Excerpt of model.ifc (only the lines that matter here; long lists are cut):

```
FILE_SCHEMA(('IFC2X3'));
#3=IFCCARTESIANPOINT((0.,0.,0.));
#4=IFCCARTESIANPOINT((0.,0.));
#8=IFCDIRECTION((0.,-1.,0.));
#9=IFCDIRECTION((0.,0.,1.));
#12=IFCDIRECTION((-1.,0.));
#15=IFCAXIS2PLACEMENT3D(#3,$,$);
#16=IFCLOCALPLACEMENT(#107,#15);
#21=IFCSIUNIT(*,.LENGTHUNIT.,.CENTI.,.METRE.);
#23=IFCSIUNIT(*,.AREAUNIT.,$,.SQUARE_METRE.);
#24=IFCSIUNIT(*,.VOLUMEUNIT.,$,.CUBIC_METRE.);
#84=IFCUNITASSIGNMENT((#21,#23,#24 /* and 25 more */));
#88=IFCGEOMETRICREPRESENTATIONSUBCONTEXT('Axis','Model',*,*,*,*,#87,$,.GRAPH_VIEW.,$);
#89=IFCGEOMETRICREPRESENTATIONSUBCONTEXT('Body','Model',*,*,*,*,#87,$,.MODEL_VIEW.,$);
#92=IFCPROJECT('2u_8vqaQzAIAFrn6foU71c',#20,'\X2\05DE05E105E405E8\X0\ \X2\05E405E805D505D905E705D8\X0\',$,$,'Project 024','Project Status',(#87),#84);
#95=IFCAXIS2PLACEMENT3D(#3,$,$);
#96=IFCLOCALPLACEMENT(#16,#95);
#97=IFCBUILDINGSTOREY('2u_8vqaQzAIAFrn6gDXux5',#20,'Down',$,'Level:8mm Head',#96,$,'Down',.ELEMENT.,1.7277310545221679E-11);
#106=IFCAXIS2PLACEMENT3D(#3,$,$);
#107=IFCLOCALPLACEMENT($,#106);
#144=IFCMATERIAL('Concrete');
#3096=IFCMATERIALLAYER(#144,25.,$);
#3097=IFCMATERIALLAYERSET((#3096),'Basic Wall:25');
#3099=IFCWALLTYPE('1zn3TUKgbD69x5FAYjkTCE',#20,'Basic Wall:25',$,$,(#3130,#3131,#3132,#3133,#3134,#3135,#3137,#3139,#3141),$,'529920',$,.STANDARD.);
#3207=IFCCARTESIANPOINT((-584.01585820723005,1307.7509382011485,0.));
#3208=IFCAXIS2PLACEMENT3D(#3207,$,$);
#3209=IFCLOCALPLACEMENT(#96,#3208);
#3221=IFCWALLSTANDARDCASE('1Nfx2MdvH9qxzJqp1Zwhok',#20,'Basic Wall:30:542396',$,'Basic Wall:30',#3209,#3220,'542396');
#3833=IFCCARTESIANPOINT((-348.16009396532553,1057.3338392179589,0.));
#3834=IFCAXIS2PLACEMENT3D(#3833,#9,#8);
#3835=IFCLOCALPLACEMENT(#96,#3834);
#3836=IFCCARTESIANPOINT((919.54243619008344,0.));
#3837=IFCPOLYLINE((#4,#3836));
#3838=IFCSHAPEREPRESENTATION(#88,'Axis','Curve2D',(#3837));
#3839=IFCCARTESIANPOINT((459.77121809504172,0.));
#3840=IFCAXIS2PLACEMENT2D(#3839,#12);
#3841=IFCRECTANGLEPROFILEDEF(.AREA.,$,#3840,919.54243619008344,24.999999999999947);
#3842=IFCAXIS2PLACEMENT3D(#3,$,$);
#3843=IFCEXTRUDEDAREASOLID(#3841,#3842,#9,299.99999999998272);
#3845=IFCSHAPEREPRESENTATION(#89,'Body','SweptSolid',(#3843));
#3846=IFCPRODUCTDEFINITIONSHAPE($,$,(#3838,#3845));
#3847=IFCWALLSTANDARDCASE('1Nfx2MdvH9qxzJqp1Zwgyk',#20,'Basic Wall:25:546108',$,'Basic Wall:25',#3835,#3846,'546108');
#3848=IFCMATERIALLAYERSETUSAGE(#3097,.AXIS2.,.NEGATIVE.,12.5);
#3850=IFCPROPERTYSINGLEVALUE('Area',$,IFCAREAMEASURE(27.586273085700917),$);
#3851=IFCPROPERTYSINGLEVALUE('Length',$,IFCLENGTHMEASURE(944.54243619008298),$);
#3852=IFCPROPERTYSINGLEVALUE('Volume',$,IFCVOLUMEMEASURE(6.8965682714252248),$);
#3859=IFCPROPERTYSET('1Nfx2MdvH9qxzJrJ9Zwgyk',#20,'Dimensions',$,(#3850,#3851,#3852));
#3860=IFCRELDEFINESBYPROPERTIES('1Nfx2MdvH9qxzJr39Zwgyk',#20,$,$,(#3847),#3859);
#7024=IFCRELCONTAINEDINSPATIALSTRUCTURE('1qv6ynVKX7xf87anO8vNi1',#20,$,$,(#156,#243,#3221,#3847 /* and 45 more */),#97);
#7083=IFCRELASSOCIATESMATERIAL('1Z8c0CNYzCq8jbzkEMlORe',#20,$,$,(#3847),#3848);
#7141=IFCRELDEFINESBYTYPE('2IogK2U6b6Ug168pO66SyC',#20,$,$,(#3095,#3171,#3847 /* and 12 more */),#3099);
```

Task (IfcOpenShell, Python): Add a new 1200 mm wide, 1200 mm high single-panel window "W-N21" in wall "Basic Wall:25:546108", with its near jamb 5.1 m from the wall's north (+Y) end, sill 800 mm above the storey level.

```python
import numpy as np
import ifcopenshell
import ifcopenshell.api.feature
import ifcopenshell.api.geometry
import ifcopenshell.api.pset
import ifcopenshell.api.root
import ifcopenshell.api.spatial
import ifcopenshell.api.type
import ifcopenshell.geom
import ifcopenshell.util.element
import ifcopenshell.util.placement
import ifcopenshell.util.representation
import ifcopenshell.util.shape
import ifcopenshell.util.unit

model = ifcopenshell.open("model.ifc")
unit_scale = ifcopenshell.util.unit.calculate_unit_scale(model)
area_scale = ifcopenshell.util.unit.calculate_unit_scale(model, "AREAUNIT")
volume_scale = ifcopenshell.util.unit.calculate_unit_scale(model, "VOLUMEUNIT")
settings = ifcopenshell.geom.settings()


def volume(element):
    """Net volume in cubic metres, openings subtracted."""
    shape = ifcopenshell.geom.create_shape(settings, element)
    return ifcopenshell.util.shape.get_volume(shape.geometry)


wall = model.by_guid("1Nfx2MdvH9qxzJqp1Zwgyk")
storey = ifcopenshell.util.element.get_container(wall, ifc_class="IfcBuildingStorey")
context = ifcopenshell.util.representation.get_context(model, "Model", "Body", "MODEL_VIEW")
before = volume(wall)

width, height, from_end, sill = 1.2, 1.2, 5.1, 0.8  # metres

# The wall runs along its own X axis, and the end named is its -X end.
wall_shape = ifcopenshell.geom.create_shape(settings, wall)
x, y, z = ifcopenshell.util.shape.get_vertices(wall_shape.geometry).T
start = x.min() + from_end
face, thickness = float(y.min()), float(y.max() - y.min())
wall_matrix = ifcopenshell.util.placement.get_local_placement(wall.ObjectPlacement)
level = ifcopenshell.util.placement.get_local_placement(storey.ObjectPlacement)[2, 3]


def in_wall(x, y):
    """Placement at x, y metres in the wall's axes, at sill height."""
    matrix = wall_matrix.copy()
    matrix[:, 3] = wall_matrix @ np.array([x / unit_scale, y / unit_scale, 0.0, 1.0])
    matrix[2, 3] = level + sill / unit_scale
    return matrix


# Opening: a box that overshoots both wall faces by 50 mm.
opening = ifcopenshell.api.root.create_entity(model, ifc_class="IfcOpeningElement")
box = ifcopenshell.api.geometry.add_wall_representation(
    model, context=context, length=width, height=height, thickness=thickness + 0.1
)
ifcopenshell.api.geometry.assign_representation(model, product=opening, representation=box)
ifcopenshell.api.geometry.edit_object_placement(model, product=opening, matrix=in_wall(start, face - 0.05), is_si=False)
ifcopenshell.api.feature.add_feature(model, feature=opening, element=wall)

window = ifcopenshell.api.root.create_entity(model, ifc_class="IfcWindow", name="W-N21")
window.OverallWidth, window.OverallHeight = width / unit_scale, height / unit_scale
body = ifcopenshell.api.geometry.add_window_representation(
    model,
    context=context,
    overall_width=window.OverallWidth,
    overall_height=window.OverallHeight,
    partition_type="SINGLE_PANEL",
)
ifcopenshell.api.geometry.assign_representation(model, product=window, representation=body)
ifcopenshell.api.spatial.assign_container(model, products=[window], relating_structure=storey)
fills = ifcopenshell.api.feature.add_filling(model, opening=opening, element=window)
fills.OwnerHistory = window.OwnerHistory  # required in IFC2X3

# IFC2X3 keeps the operation on the window style.
style = ifcopenshell.api.root.create_entity(model, ifc_class="IfcWindowStyle", name="W-N21")
style.OperationType, style.ConstructionType = "SINGLE_PANEL", "NOTDEFINED"
style.ParameterTakesPrecedence = style.Sizeable = False
ifcopenshell.api.type.assign_type(model, related_objects=[window], relating_type=style)

# Centre the window in the wall's thickness.
ifcopenshell.api.geometry.edit_object_placement(model, product=window, matrix=in_wall(start, face), is_si=False)
window_shape = ifcopenshell.geom.create_shape(settings, window)
depth = ifcopenshell.util.shape.get_vertices(window_shape.geometry)[:, 1]
offset = face + thickness / 2 - (depth.min() + depth.max()) / 2
ifcopenshell.api.geometry.edit_object_placement(model, product=window, matrix=in_wall(start, offset), is_si=False)

after = volume(wall)

# Update the wall's stored quantities.
pset = model.by_id(ifcopenshell.util.element.get_pset(wall, "Dimensions", should_inherit=False)["id"])
ifcopenshell.api.pset.edit_pset(model, pset=pset, properties={
    "Area": model.create_entity("IfcAreaMeasure", after / thickness / area_scale),
    "Volume": model.create_entity("IfcVolumeMeasure", after / volume_scale),
})

print(f"wall volume {before:.3f} -> {after:.3f} m3")

model.write("model_edited.ifc")
```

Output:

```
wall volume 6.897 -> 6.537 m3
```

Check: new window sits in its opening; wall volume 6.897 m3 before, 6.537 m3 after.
